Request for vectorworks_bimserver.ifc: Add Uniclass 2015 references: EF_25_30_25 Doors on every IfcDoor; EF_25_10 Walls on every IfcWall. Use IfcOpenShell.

First a look at what the model holds.

```python
import ifcopenshell

model = ifcopenshell.open("vectorworks_bimserver.ifc")
print(model.schema)
print("classifications:", [c.Name for c in model.by_type("IfcClassification")])
for ifc_class in ("IfcDoor", "IfcRoof", "IfcStair", "IfcWall", "IfcWindow"):
    print(ifc_class, len(model.by_type(ifc_class)))
```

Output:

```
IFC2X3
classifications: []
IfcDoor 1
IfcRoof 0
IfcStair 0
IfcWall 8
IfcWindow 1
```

```python
import ifcopenshell
import ifcopenshell.api.classification

model = ifcopenshell.open("vectorworks_bimserver.ifc")

# IFC2X3 requires Source and Edition and has no link from the project to the system.
system = model.create_entity("IfcClassification", Source="NBS", Edition="2015", Name="Uniclass 2015")

codes = {
    "IfcDoor": ("EF_25_30_25", "Doors"),
    "IfcWall": ("EF_25_10", "Walls"),
}
for ifc_class, (code, name) in codes.items():
    products = model.by_type(ifc_class)
    ifcopenshell.api.classification.add_reference(
        model, products=products, classification=system, identification=code, name=name
    )
    print(code, len(products))

model.write("vectorworks_bimserver_v2.ifc")
```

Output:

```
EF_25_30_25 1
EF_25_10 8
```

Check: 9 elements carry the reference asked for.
